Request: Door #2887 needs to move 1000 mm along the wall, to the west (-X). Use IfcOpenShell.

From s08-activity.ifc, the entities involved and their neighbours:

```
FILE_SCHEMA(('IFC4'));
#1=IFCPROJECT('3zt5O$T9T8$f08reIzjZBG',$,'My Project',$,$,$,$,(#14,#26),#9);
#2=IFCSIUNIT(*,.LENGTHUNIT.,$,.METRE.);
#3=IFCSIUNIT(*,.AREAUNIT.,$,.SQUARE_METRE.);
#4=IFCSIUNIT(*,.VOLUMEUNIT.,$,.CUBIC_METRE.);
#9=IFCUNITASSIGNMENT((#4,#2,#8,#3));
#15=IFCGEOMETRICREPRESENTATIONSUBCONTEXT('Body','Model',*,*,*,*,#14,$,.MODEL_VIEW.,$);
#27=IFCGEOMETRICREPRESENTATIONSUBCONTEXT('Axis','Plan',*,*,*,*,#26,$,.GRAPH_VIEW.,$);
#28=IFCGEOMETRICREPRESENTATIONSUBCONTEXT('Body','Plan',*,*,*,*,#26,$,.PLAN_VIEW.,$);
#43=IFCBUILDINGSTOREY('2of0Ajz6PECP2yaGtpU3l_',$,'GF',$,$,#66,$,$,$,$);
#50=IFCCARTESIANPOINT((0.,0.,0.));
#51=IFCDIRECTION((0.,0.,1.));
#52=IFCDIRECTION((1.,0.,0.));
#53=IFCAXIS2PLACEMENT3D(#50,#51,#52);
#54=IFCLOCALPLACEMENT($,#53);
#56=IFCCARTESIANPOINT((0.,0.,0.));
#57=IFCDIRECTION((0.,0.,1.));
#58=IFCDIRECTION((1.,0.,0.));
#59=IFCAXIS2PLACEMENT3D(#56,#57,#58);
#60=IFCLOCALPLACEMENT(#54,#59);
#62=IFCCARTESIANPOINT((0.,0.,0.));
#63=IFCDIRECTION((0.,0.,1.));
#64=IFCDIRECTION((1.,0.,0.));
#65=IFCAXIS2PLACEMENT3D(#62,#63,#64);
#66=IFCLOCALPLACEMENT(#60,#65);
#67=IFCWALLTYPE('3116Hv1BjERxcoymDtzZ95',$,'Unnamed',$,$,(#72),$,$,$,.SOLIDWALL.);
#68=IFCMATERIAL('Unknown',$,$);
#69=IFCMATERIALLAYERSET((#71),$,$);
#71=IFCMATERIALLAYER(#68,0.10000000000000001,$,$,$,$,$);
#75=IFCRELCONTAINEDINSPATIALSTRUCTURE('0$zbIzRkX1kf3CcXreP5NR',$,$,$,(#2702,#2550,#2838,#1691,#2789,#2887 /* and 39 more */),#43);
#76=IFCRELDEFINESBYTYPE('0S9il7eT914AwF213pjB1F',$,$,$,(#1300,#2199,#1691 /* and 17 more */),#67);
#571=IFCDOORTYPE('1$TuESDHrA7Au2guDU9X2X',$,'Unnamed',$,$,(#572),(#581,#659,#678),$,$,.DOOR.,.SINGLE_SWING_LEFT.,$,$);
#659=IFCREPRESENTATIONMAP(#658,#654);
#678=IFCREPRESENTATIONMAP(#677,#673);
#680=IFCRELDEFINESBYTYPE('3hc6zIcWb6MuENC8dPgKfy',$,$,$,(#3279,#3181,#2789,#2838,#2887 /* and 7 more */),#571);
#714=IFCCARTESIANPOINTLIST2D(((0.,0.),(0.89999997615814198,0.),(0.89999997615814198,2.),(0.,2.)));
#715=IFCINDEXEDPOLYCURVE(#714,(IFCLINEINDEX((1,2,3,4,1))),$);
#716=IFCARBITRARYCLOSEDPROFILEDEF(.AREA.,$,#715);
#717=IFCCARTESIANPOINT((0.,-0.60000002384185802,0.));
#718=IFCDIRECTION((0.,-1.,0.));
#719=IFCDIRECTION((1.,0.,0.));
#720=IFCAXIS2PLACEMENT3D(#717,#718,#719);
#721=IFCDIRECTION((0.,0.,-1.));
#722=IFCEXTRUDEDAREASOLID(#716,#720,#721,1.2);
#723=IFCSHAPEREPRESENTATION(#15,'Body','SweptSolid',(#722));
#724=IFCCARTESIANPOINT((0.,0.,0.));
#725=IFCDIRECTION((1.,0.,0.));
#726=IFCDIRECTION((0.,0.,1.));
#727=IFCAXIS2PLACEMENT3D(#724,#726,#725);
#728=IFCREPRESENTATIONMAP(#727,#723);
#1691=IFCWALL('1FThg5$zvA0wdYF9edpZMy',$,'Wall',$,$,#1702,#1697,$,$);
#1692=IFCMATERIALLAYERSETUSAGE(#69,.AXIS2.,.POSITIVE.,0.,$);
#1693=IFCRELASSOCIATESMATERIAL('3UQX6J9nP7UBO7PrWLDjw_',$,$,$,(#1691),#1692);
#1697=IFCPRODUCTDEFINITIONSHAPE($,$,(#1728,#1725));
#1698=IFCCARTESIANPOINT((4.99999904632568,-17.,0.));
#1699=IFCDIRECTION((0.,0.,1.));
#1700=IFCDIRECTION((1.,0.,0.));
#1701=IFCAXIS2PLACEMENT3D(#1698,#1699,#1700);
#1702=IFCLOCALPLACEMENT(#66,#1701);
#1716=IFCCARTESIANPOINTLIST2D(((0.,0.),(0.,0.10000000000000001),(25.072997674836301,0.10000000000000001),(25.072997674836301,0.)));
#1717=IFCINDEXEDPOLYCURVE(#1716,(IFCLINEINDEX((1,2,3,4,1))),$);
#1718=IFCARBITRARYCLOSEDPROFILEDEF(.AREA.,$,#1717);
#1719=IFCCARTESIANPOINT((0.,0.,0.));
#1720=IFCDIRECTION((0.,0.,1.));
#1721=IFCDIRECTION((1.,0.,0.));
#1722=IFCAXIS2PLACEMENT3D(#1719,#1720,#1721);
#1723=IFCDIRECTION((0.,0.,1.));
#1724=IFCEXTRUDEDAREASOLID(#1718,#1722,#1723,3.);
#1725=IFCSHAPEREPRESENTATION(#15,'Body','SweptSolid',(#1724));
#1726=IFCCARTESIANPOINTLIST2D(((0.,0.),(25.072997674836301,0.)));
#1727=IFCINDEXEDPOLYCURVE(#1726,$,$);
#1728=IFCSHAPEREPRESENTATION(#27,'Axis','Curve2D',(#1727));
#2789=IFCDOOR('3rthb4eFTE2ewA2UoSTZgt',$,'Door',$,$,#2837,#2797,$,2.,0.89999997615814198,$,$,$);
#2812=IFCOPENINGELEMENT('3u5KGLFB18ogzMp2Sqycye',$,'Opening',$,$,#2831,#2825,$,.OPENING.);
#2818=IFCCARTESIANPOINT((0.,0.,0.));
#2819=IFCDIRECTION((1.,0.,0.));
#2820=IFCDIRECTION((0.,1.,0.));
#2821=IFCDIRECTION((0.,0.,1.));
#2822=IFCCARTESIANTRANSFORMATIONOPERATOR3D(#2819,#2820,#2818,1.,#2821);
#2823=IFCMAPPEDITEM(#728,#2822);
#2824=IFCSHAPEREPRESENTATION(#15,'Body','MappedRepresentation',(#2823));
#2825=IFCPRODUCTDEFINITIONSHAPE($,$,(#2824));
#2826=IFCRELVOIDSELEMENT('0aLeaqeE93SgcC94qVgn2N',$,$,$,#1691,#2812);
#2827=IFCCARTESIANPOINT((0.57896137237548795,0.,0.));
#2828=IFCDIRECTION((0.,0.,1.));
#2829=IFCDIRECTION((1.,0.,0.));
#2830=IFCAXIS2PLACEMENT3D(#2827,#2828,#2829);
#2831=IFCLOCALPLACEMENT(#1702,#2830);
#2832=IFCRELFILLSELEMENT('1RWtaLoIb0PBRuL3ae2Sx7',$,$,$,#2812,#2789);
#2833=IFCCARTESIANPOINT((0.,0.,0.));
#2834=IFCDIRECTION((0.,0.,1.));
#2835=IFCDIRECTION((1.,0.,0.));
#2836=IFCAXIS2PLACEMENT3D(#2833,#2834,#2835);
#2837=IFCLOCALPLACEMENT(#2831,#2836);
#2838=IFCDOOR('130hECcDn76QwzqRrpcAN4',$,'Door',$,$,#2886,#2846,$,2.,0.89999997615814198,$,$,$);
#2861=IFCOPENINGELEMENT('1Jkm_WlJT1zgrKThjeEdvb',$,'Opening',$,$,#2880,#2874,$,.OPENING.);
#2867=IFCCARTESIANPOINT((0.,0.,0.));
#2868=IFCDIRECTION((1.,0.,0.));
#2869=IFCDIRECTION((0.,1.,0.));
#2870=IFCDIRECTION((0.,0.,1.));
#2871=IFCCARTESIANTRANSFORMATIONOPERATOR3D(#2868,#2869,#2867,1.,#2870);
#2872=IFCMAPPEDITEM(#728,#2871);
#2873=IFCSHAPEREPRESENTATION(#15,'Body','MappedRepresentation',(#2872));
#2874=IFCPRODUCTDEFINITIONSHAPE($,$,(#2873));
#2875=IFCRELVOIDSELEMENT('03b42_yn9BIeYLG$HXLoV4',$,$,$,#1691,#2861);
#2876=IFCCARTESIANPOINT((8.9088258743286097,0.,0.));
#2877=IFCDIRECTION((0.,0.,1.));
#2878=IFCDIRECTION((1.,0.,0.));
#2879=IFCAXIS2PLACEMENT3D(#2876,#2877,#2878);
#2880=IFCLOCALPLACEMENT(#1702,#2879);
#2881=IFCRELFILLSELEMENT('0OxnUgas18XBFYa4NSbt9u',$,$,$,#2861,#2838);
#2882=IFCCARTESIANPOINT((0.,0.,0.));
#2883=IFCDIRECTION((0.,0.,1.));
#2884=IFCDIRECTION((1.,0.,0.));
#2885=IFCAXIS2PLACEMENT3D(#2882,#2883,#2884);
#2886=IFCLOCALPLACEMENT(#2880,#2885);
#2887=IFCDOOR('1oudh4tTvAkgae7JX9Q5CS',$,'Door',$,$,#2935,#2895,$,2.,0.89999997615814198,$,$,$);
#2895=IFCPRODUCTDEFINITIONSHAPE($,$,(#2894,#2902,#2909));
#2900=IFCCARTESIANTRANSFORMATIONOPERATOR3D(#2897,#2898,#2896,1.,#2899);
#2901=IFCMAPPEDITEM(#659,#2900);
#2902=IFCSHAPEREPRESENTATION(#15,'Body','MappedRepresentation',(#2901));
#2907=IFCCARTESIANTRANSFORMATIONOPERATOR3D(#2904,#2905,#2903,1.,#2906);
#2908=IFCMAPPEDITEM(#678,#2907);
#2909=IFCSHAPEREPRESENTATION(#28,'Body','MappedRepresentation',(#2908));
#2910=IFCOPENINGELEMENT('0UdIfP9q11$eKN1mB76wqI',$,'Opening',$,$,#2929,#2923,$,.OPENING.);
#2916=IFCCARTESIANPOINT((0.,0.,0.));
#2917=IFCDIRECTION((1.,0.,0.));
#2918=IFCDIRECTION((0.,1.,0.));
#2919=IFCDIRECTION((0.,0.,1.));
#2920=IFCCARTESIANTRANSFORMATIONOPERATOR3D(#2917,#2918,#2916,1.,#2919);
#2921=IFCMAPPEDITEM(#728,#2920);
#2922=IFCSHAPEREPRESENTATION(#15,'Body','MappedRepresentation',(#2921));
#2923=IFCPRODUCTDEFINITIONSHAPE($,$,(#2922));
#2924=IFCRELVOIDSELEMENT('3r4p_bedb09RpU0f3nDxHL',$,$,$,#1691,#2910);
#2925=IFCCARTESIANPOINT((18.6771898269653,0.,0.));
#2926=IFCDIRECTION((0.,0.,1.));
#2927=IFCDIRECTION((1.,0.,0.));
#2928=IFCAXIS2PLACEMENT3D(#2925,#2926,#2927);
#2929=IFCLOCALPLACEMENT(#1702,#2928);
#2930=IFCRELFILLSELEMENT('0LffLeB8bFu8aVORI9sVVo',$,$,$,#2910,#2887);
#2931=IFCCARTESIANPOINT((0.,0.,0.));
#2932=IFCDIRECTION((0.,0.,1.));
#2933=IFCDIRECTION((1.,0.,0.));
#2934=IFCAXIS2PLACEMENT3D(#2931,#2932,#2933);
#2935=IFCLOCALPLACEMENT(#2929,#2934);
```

```python
import ifcopenshell
import ifcopenshell.api.geometry
import ifcopenshell.util.placement
import ifcopenshell.util.unit

model = ifcopenshell.open("s08-activity.ifc")
unit_scale = ifcopenshell.util.unit.calculate_unit_scale(model)

door = model.by_guid("1oudh4tTvAkgae7JX9Q5CS")
opening = door.FillsVoids[0].RelatingOpeningElement
wall = opening.VoidsElements[0].RelatingBuildingElement

wall_matrix = ifcopenshell.util.placement.get_local_placement(wall.ObjectPlacement)
shift = wall_matrix[:3, 0] * -1 / unit_scale
before = ifcopenshell.util.placement.get_local_placement(door.ObjectPlacement)[:3, 3].copy()

# The door is placed relative to its opening, so it follows when the opening moves.
matrix = ifcopenshell.util.placement.get_local_placement(opening.ObjectPlacement)
matrix[:3, 3] += shift
ifcopenshell.api.geometry.edit_object_placement(
    model, product=opening, matrix=matrix, is_si=False, should_transform_children=True
)

after = ifcopenshell.util.placement.get_local_placement(door.ObjectPlacement)[:3, 3]
print("door moved by", (after - before).round(3) + 0.0)

model.write("s08-activity_rev.ifc")
```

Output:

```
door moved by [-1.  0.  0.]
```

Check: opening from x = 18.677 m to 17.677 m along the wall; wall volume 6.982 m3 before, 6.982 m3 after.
